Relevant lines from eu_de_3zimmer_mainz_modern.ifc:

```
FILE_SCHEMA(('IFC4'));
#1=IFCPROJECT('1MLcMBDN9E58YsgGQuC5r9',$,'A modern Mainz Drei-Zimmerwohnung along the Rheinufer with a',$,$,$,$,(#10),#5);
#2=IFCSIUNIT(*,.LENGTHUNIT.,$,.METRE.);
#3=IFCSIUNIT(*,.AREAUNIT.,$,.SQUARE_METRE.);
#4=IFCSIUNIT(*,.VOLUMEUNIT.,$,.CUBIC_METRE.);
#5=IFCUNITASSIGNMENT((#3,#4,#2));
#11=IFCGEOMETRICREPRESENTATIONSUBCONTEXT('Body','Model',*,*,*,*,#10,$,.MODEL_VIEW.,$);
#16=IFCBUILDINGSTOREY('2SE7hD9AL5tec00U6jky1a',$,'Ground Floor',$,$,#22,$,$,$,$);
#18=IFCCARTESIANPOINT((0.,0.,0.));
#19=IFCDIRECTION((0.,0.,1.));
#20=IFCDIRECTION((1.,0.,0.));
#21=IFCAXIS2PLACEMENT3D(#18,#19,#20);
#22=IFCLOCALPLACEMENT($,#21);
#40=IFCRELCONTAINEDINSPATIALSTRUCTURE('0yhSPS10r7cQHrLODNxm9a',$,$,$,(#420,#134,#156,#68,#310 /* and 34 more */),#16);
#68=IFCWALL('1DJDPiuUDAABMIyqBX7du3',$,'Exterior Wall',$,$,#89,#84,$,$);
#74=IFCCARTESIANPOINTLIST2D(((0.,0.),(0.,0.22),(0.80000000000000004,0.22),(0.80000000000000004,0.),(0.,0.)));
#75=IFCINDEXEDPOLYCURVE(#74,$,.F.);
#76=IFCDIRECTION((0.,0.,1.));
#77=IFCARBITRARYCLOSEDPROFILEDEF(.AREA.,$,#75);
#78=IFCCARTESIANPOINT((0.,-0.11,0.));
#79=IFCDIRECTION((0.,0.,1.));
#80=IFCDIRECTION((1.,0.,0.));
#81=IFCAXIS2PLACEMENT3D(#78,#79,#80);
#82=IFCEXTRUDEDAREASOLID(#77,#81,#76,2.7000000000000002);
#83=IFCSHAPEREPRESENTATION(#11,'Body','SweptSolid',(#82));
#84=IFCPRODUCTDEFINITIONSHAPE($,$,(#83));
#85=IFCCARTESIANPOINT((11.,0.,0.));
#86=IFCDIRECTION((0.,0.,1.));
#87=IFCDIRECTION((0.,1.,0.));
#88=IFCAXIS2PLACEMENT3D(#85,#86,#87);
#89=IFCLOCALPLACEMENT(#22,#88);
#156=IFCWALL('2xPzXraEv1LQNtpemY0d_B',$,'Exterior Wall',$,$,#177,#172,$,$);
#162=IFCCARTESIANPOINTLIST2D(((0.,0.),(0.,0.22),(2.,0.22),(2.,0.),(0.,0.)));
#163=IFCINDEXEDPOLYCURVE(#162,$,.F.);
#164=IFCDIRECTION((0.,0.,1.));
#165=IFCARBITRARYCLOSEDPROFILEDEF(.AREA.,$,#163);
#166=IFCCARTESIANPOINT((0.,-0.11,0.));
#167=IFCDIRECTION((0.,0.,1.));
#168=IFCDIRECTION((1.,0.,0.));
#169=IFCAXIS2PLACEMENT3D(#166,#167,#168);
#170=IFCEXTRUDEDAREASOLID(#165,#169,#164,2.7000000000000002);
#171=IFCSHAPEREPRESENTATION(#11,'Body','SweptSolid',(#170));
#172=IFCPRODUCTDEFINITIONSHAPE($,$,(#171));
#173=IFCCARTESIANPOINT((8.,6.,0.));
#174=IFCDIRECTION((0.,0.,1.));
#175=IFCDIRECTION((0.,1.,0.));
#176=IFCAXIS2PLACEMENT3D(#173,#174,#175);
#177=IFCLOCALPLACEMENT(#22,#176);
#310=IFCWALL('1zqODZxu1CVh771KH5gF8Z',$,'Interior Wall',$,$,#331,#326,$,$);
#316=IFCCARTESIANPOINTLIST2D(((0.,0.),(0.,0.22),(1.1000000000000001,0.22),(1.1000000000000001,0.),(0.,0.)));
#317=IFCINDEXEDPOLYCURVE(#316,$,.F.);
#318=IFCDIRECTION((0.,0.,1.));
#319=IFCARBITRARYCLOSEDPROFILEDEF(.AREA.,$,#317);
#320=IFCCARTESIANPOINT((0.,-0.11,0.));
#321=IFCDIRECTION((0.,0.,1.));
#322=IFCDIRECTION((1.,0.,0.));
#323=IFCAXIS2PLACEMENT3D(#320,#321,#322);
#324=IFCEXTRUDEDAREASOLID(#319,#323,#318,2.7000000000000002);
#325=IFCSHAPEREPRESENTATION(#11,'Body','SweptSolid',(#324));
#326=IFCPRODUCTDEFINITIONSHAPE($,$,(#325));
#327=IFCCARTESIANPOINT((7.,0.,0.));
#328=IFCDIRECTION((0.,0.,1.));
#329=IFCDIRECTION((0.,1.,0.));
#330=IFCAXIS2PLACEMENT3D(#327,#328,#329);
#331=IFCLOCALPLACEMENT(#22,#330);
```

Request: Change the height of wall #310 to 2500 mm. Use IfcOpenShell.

```python
import ifcopenshell
import ifcopenshell.geom
import ifcopenshell.util.representation
import ifcopenshell.util.shape
import ifcopenshell.util.unit

model = ifcopenshell.open("eu_de_3zimmer_mainz_modern.ifc")
unit_scale = ifcopenshell.util.unit.calculate_unit_scale(model)
settings = ifcopenshell.geom.settings()


def volume(element):
    """Net volume in cubic metres, openings subtracted."""
    shape = ifcopenshell.geom.create_shape(settings, element)
    return ifcopenshell.util.shape.get_volume(shape.geometry)


wall = model.by_guid("1zqODZxu1CVh771KH5gF8Z")
before = volume(wall)

body = ifcopenshell.util.representation.get_representation(wall, "Model", "Body")
solid = body.Items[0]
old_height = solid.Depth
solid.Depth = 2.5 / unit_scale
after = volume(wall)

print(f"height {old_height:g} -> {solid.Depth:g}, volume {before:.3f} -> {after:.3f} m3")

model.write("eu_de_3zimmer_mainz_modern_v2.ifc")
```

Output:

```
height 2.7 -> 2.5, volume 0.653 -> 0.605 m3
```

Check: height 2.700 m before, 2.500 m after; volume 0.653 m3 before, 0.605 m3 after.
